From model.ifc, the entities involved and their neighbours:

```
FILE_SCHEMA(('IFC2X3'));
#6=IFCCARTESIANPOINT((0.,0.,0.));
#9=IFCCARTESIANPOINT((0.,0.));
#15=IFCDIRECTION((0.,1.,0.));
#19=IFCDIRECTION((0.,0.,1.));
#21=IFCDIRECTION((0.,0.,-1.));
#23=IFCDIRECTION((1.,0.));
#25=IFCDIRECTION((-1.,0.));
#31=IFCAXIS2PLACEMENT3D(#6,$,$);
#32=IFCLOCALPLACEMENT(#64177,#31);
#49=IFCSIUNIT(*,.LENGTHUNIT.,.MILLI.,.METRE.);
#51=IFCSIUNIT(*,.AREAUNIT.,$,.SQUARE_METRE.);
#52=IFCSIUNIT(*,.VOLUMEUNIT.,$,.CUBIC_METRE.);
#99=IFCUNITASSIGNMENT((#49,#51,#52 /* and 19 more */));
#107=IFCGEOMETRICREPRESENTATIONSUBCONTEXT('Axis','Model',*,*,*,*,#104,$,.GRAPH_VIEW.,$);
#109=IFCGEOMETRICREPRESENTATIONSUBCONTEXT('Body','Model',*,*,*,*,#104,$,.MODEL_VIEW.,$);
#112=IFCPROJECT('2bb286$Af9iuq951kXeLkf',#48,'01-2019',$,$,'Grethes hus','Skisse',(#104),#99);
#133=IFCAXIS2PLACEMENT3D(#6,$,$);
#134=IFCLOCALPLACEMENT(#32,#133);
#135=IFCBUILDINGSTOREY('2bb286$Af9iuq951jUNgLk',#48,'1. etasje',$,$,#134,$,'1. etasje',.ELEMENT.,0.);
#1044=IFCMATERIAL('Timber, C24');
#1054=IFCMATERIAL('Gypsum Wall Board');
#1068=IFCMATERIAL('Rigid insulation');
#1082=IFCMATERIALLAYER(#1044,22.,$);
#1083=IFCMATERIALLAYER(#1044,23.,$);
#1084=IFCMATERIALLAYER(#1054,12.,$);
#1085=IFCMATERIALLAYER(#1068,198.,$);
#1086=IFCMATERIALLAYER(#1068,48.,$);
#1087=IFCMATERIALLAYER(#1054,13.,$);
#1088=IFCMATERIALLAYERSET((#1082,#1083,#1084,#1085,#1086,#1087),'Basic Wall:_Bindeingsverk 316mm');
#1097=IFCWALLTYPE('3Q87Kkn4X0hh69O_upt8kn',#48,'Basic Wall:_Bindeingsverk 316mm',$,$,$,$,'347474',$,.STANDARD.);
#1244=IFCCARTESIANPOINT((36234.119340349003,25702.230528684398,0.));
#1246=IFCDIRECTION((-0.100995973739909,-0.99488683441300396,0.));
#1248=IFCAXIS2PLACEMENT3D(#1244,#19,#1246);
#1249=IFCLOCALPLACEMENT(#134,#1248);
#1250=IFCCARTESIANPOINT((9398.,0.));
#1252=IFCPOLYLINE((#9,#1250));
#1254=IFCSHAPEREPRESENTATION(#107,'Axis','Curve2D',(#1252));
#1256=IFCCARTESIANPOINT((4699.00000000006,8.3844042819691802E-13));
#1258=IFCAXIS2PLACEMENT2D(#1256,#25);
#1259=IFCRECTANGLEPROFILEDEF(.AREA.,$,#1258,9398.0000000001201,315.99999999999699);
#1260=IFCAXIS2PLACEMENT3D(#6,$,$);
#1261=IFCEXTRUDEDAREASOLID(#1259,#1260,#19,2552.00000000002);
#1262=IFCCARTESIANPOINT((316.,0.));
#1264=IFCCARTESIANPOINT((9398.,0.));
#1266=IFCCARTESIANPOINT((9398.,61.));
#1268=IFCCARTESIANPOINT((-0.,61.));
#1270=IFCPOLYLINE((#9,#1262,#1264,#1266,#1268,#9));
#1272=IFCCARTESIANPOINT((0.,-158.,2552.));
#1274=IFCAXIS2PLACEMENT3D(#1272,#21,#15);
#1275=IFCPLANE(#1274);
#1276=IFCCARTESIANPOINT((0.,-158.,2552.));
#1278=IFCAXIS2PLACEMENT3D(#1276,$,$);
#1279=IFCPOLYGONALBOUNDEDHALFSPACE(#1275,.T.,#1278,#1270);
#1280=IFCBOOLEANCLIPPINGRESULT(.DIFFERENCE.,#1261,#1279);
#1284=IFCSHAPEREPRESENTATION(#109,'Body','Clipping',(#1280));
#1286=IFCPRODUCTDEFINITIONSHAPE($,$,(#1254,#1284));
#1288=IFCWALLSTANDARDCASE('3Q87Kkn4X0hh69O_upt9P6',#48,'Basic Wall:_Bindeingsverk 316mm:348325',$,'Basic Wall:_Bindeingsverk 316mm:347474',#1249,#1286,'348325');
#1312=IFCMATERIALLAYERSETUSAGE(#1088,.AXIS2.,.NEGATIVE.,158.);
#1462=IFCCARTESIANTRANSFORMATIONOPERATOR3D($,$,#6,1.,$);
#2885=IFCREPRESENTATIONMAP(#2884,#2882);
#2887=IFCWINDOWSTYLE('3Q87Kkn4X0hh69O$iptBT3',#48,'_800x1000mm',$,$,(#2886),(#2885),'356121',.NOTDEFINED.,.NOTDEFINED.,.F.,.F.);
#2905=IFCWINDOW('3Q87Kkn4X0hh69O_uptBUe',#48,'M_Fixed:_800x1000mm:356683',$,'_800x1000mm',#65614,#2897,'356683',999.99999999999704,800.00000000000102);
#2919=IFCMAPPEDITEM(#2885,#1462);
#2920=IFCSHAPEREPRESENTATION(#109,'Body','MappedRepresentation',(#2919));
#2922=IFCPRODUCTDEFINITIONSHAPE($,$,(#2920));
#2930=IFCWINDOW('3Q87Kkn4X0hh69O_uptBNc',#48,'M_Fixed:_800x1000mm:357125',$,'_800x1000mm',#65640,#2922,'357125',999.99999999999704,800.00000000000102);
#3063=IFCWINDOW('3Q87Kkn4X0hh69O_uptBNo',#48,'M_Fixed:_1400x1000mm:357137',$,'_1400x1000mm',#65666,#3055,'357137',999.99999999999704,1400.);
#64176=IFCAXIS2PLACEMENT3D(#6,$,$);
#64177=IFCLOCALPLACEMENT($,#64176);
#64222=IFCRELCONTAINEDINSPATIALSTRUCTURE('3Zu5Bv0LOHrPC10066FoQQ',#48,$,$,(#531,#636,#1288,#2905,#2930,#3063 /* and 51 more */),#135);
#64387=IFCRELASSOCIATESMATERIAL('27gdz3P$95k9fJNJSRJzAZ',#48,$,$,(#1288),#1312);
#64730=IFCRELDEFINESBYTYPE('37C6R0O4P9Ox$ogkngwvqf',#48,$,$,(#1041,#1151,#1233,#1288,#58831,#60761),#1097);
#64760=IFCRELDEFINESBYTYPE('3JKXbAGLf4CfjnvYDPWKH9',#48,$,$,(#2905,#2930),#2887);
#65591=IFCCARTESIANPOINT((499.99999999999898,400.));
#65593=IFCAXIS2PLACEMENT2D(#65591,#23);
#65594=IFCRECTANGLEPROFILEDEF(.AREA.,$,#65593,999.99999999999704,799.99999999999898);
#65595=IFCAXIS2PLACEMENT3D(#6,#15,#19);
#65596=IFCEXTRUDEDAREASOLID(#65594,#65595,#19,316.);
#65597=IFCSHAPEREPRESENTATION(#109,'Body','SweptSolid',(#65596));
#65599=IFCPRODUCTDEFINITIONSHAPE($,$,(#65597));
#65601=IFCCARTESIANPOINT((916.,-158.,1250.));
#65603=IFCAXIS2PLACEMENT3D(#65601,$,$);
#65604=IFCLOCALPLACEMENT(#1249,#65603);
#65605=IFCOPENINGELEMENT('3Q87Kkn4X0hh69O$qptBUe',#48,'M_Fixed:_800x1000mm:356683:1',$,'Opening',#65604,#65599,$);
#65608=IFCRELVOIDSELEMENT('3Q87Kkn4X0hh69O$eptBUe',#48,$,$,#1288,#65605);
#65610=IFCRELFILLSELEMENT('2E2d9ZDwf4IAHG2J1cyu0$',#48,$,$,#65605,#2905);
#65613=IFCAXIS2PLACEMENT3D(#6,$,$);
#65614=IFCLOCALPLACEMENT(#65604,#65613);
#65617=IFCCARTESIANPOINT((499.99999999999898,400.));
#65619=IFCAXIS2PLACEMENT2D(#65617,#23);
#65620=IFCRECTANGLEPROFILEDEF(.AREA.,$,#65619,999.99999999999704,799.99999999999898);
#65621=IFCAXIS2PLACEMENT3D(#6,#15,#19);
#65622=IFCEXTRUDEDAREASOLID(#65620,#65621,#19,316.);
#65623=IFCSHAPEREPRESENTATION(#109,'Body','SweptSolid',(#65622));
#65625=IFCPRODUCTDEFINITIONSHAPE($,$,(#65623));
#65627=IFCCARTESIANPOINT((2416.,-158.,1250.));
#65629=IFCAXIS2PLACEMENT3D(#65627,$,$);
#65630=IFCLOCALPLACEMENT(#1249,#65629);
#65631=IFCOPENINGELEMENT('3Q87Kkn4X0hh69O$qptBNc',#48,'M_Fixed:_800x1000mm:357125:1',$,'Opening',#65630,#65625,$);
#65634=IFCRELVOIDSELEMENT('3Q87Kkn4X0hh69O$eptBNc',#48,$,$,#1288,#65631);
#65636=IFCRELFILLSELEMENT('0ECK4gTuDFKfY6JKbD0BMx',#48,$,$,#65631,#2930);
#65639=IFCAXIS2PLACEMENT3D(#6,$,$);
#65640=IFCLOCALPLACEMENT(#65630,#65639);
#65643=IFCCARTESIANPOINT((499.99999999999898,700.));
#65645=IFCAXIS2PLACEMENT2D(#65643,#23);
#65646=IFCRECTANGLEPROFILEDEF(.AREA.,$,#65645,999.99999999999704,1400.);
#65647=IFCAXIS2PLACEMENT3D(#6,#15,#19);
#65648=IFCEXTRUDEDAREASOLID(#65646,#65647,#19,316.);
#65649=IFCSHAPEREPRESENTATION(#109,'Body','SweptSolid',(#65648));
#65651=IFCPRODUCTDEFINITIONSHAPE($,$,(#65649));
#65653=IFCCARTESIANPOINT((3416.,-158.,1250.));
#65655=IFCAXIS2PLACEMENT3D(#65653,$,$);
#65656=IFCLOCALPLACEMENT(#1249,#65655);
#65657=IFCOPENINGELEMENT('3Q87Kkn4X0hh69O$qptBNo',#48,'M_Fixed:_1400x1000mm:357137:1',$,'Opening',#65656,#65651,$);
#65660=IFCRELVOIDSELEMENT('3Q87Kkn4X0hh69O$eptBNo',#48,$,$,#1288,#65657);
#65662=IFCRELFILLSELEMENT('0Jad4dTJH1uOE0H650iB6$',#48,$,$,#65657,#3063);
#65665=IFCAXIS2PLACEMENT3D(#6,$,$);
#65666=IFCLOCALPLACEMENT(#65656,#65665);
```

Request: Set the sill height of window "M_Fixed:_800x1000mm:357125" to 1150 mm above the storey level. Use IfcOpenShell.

```python
import numpy as np
import ifcopenshell
import ifcopenshell.api.geometry
import ifcopenshell.geom
import ifcopenshell.util.element
import ifcopenshell.util.placement
import ifcopenshell.util.shape
import ifcopenshell.util.unit

model = ifcopenshell.open("model.ifc")
unit_scale = ifcopenshell.util.unit.calculate_unit_scale(model)

window = model.by_guid("3Q87Kkn4X0hh69O_uptBNc")
opening = window.FillsVoids[0].RelatingOpeningElement
storey = ifcopenshell.util.element.get_container(window, ifc_class="IfcBuildingStorey")
level = ifcopenshell.util.placement.get_local_placement(storey.ObjectPlacement)[2, 3]

# The opening's origin need not be at the sill, so measure its lowest point.
shape = ifcopenshell.geom.create_shape(ifcopenshell.geom.settings(), opening)
bottom = ifcopenshell.util.shape.get_shape_bottom_elevation(shape, shape.geometry) / unit_scale
dz = level + 1150.0 - bottom

shift = np.array([0.0, 0.0, dz])
# The window is placed relative to its opening, so it follows when the opening moves.
matrix = ifcopenshell.util.placement.get_local_placement(opening.ObjectPlacement)
matrix[:3, 3] += shift
ifcopenshell.api.geometry.edit_object_placement(
    model, product=opening, matrix=matrix, is_si=False, should_transform_children=True
)

print(f"moved by {dz * unit_scale:+.3f} m")

model.write("model_rev.ifc")
```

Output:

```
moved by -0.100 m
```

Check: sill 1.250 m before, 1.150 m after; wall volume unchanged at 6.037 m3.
